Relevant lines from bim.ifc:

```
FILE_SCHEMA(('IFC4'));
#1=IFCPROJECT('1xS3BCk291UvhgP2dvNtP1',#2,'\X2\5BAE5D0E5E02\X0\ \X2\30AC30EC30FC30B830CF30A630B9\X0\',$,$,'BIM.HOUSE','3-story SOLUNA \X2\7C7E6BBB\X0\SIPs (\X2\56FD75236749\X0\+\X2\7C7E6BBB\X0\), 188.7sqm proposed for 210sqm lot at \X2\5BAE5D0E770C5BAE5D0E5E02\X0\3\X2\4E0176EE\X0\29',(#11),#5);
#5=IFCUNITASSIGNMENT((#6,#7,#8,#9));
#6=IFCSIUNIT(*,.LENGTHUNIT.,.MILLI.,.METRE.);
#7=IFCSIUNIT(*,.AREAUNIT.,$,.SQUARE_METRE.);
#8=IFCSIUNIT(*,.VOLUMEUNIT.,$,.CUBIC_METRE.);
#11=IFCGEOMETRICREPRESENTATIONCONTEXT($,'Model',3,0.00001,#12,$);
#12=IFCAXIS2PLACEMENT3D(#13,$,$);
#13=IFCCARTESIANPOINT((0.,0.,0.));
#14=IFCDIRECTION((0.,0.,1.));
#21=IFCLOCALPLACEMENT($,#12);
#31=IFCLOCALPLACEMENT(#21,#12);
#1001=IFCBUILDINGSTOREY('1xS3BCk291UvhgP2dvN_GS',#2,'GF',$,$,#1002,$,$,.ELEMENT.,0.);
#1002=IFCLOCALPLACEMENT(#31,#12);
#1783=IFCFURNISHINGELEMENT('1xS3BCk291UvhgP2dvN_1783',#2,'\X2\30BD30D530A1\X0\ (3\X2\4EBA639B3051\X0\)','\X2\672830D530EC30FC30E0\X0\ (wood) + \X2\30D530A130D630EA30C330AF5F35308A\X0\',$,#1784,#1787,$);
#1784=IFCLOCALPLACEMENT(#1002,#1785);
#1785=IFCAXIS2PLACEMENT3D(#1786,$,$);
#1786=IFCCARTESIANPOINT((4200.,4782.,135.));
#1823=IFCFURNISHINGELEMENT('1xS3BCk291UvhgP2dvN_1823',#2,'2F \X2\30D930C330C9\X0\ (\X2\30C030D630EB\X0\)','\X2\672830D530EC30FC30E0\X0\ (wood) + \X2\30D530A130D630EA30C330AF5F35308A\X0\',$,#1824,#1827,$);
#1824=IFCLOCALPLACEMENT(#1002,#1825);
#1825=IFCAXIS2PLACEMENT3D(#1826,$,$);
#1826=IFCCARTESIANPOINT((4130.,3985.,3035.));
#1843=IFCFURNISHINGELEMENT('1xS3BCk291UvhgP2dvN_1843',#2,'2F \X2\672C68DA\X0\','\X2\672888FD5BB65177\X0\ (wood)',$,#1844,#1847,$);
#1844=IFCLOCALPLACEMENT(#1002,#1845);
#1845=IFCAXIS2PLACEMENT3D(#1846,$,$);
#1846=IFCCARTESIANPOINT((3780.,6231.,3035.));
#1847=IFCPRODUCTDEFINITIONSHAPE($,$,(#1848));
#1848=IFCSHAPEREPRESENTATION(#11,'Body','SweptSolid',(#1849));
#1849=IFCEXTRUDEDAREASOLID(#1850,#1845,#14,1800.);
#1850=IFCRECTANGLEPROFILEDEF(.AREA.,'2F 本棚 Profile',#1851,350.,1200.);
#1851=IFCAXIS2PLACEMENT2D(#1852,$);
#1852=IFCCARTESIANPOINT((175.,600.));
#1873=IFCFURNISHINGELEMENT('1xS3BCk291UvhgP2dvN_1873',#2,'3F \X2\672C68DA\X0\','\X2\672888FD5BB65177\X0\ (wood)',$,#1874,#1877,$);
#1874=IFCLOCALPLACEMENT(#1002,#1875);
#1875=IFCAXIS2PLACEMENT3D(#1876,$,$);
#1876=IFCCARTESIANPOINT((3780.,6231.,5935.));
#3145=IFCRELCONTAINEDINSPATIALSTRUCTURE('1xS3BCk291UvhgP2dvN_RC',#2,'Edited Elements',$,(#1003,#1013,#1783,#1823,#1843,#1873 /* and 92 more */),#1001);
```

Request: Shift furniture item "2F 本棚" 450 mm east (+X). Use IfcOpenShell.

```python
import ifcopenshell
import ifcopenshell.api.geometry
import ifcopenshell.util.placement

model = ifcopenshell.open("bim.ifc")

item = model.by_id(1843)
matrix = ifcopenshell.util.placement.get_local_placement(item.ObjectPlacement)
matrix[0, 3] += 450.0
ifcopenshell.api.geometry.edit_object_placement(model, product=item, matrix=matrix, is_si=False)

print(ifcopenshell.util.placement.get_local_placement(item.ObjectPlacement).round(3) + 0.0)

model.write("bim_v2.ifc")
```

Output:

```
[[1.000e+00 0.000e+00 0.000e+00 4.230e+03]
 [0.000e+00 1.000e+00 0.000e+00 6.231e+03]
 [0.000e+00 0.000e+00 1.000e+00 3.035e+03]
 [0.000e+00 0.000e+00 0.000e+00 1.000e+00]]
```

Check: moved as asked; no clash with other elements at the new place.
